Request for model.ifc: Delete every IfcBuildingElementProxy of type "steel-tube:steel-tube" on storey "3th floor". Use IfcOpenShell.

First a look at what the model holds.

```python
import ifcopenshell
import ifcopenshell.util.element

model = ifcopenshell.open("model.ifc")
print(model.schema)
storey = next(s for s in model.by_type("IfcBuildingStorey") if s.Name == "3th floor")
proxies = [e for e in ifcopenshell.util.element.get_decomposition(storey) if e.is_a("IfcBuildingElementProxy")]
seen = {}
for e in proxies:
    element_type = ifcopenshell.util.element.get_type(e)
    name = element_type.Name if element_type not in (None, e) else None
    seen[name] = seen.get(name, 0) + 1
for name, count in sorted(seen.items(), key=str):
    print(count, "x", name)
```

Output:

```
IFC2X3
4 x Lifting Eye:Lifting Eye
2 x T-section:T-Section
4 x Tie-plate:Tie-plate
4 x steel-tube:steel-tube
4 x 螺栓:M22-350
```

```python
import ifcopenshell
import ifcopenshell.api.root
import ifcopenshell.util.element

model = ifcopenshell.open("model.ifc")

storey = next(s for s in model.by_type("IfcBuildingStorey") if s.Name == "3th floor")
proxies = [e for e in ifcopenshell.util.element.get_decomposition(storey) if e.is_a("IfcBuildingElementProxy")]
targets = [e for e in proxies if (t := ifcopenshell.util.element.get_type(e)) not in (None, e) and t.Name == "steel-tube:steel-tube"]

for e in targets:
    ifcopenshell.api.root.remove_product(model, product=e)
print(len(targets), "removed")

model.write("model_edited.ifc")
```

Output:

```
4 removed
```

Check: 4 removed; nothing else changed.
